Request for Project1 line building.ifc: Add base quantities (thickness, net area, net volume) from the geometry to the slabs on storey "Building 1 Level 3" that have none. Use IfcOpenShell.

First a look at what the model holds.

```python
import ifcopenshell
import ifcopenshell.util.element
import ifcopenshell.util.unit

model = ifcopenshell.open("Project1 line building.ifc")
print(model.schema)
for unit_type in ("LENGTHUNIT", "AREAUNIT", "VOLUMEUNIT"):
    print(unit_type, ifcopenshell.util.unit.calculate_unit_scale(model, unit_type))
storey = next(s for s in model.by_type("IfcBuildingStorey") if s.Name == "Building 1 Level 3")
slabs = [e for e in ifcopenshell.util.element.get_decomposition(storey) if e.is_a("IfcSlab")]
for e in sorted(slabs, key=lambda e: e.id()):
    print(e.id(), e.is_a(), e.Name, list(ifcopenshell.util.element.get_psets(e, qtos_only=True)), sep=" | ")
```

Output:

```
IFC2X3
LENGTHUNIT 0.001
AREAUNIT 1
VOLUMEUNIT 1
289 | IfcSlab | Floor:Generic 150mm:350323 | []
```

```python
import ifcopenshell
import ifcopenshell.api.pset
import ifcopenshell.geom
import ifcopenshell.util.element
import ifcopenshell.util.shape
import ifcopenshell.util.unit

model = ifcopenshell.open("Project1 line building.ifc")
unit_scale = ifcopenshell.util.unit.calculate_unit_scale(model)
area_scale = ifcopenshell.util.unit.calculate_unit_scale(model, "AREAUNIT")
volume_scale = ifcopenshell.util.unit.calculate_unit_scale(model, "VOLUMEUNIT")
settings = ifcopenshell.geom.settings()

storey = next(s for s in model.by_type("IfcBuildingStorey") if s.Name == "Building 1 Level 3")
slabs = [e for e in ifcopenshell.util.element.get_decomposition(storey) if e.is_a("IfcSlab")]

for e in sorted(slabs, key=lambda e: e.id()):
    if ifcopenshell.util.element.get_psets(e, qtos_only=True, should_inherit=False):
        continue
    # Geometry comes back in metres, in the element's own axes.
    shape = ifcopenshell.geom.create_shape(settings, e)
    values = {
        "Width": ifcopenshell.util.shape.get_z(shape.geometry) / unit_scale,
        "NetArea": ifcopenshell.util.shape.get_footprint_area(shape.geometry) / area_scale,
        "NetVolume": ifcopenshell.util.shape.get_volume(shape.geometry) / volume_scale,
    }
    qto = ifcopenshell.api.pset.add_qto(model, product=e, name="BaseQuantities")
    ifcopenshell.api.pset.edit_qto(model, qto=qto, properties=values)
    print(e.id(), {k: round(v, 3) for k, v in values.items()})

model.write("Project1 line building_edited.ifc")
```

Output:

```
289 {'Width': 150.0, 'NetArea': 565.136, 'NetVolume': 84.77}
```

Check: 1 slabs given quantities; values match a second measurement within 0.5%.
